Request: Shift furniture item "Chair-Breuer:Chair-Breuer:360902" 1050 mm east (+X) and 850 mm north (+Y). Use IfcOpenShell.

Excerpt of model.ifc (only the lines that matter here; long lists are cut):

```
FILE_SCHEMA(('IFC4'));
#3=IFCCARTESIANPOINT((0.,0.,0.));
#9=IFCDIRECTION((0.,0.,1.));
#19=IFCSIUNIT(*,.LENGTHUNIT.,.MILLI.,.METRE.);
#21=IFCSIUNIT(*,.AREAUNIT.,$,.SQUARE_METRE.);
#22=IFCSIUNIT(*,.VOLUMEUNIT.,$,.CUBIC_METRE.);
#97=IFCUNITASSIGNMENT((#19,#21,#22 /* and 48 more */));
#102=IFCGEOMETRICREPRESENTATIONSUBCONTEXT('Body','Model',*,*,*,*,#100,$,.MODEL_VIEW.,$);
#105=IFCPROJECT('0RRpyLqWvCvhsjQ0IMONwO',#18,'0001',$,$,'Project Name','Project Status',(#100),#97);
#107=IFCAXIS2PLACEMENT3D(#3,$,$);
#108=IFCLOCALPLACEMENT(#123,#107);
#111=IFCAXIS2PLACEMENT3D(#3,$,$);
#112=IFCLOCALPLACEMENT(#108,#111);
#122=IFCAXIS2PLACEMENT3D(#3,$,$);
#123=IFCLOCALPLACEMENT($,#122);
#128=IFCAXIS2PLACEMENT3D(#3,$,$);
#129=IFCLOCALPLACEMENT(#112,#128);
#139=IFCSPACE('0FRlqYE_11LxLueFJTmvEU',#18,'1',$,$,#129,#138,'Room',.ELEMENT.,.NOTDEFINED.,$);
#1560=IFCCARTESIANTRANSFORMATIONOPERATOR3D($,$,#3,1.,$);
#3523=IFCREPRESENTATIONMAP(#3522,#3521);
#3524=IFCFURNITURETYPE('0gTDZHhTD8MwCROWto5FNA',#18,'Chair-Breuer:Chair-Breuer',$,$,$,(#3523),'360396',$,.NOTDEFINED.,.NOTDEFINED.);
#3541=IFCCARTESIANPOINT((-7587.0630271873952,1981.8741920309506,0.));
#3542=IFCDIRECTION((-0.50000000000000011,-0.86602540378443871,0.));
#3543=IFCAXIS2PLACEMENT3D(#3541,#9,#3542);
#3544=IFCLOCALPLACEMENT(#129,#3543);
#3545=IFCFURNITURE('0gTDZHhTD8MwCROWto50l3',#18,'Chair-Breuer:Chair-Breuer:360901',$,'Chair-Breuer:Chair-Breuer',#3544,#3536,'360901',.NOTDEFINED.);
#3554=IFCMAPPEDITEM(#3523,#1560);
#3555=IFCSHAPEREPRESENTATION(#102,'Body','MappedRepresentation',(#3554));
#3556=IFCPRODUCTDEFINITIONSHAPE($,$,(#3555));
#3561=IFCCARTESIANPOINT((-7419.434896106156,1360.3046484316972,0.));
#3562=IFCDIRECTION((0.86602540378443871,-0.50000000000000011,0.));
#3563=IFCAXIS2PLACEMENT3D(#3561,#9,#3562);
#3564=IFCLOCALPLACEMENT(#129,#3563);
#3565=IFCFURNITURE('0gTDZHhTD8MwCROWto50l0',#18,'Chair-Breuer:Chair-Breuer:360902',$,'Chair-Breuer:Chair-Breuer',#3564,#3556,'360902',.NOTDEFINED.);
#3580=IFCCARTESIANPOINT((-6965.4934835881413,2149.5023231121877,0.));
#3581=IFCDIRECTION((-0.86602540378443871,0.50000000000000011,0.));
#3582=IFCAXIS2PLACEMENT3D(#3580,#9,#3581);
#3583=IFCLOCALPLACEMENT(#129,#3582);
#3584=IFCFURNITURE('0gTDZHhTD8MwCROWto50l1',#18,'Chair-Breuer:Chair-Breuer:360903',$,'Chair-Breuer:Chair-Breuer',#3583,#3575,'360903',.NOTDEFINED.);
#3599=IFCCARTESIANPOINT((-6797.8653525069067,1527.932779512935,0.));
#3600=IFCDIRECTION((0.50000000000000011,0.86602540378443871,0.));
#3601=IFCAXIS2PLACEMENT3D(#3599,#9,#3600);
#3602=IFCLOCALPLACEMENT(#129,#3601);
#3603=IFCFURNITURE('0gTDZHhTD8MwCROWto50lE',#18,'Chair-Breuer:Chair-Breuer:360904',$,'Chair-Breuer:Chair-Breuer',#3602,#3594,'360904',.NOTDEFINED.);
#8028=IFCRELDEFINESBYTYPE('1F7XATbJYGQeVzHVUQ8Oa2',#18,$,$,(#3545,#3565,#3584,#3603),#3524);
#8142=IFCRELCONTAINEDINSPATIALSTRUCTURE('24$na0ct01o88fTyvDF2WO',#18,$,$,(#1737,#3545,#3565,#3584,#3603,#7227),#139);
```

```python
import ifcopenshell
import ifcopenshell.api.geometry
import ifcopenshell.util.placement

model = ifcopenshell.open("model.ifc")

item = model.by_guid("0gTDZHhTD8MwCROWto50l0")
matrix = ifcopenshell.util.placement.get_local_placement(item.ObjectPlacement)
matrix[0, 3] += 1050.0
matrix[1, 3] += 850.0
ifcopenshell.api.geometry.edit_object_placement(model, product=item, matrix=matrix, is_si=False)

print(ifcopenshell.util.placement.get_local_placement(item.ObjectPlacement).round(3) + 0.0)

model.write("model_rev.ifc")
```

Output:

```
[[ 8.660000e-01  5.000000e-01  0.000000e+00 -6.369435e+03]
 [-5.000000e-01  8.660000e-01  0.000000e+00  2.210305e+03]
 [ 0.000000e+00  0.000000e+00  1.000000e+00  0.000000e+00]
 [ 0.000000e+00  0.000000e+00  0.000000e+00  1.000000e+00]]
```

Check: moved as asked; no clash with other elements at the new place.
